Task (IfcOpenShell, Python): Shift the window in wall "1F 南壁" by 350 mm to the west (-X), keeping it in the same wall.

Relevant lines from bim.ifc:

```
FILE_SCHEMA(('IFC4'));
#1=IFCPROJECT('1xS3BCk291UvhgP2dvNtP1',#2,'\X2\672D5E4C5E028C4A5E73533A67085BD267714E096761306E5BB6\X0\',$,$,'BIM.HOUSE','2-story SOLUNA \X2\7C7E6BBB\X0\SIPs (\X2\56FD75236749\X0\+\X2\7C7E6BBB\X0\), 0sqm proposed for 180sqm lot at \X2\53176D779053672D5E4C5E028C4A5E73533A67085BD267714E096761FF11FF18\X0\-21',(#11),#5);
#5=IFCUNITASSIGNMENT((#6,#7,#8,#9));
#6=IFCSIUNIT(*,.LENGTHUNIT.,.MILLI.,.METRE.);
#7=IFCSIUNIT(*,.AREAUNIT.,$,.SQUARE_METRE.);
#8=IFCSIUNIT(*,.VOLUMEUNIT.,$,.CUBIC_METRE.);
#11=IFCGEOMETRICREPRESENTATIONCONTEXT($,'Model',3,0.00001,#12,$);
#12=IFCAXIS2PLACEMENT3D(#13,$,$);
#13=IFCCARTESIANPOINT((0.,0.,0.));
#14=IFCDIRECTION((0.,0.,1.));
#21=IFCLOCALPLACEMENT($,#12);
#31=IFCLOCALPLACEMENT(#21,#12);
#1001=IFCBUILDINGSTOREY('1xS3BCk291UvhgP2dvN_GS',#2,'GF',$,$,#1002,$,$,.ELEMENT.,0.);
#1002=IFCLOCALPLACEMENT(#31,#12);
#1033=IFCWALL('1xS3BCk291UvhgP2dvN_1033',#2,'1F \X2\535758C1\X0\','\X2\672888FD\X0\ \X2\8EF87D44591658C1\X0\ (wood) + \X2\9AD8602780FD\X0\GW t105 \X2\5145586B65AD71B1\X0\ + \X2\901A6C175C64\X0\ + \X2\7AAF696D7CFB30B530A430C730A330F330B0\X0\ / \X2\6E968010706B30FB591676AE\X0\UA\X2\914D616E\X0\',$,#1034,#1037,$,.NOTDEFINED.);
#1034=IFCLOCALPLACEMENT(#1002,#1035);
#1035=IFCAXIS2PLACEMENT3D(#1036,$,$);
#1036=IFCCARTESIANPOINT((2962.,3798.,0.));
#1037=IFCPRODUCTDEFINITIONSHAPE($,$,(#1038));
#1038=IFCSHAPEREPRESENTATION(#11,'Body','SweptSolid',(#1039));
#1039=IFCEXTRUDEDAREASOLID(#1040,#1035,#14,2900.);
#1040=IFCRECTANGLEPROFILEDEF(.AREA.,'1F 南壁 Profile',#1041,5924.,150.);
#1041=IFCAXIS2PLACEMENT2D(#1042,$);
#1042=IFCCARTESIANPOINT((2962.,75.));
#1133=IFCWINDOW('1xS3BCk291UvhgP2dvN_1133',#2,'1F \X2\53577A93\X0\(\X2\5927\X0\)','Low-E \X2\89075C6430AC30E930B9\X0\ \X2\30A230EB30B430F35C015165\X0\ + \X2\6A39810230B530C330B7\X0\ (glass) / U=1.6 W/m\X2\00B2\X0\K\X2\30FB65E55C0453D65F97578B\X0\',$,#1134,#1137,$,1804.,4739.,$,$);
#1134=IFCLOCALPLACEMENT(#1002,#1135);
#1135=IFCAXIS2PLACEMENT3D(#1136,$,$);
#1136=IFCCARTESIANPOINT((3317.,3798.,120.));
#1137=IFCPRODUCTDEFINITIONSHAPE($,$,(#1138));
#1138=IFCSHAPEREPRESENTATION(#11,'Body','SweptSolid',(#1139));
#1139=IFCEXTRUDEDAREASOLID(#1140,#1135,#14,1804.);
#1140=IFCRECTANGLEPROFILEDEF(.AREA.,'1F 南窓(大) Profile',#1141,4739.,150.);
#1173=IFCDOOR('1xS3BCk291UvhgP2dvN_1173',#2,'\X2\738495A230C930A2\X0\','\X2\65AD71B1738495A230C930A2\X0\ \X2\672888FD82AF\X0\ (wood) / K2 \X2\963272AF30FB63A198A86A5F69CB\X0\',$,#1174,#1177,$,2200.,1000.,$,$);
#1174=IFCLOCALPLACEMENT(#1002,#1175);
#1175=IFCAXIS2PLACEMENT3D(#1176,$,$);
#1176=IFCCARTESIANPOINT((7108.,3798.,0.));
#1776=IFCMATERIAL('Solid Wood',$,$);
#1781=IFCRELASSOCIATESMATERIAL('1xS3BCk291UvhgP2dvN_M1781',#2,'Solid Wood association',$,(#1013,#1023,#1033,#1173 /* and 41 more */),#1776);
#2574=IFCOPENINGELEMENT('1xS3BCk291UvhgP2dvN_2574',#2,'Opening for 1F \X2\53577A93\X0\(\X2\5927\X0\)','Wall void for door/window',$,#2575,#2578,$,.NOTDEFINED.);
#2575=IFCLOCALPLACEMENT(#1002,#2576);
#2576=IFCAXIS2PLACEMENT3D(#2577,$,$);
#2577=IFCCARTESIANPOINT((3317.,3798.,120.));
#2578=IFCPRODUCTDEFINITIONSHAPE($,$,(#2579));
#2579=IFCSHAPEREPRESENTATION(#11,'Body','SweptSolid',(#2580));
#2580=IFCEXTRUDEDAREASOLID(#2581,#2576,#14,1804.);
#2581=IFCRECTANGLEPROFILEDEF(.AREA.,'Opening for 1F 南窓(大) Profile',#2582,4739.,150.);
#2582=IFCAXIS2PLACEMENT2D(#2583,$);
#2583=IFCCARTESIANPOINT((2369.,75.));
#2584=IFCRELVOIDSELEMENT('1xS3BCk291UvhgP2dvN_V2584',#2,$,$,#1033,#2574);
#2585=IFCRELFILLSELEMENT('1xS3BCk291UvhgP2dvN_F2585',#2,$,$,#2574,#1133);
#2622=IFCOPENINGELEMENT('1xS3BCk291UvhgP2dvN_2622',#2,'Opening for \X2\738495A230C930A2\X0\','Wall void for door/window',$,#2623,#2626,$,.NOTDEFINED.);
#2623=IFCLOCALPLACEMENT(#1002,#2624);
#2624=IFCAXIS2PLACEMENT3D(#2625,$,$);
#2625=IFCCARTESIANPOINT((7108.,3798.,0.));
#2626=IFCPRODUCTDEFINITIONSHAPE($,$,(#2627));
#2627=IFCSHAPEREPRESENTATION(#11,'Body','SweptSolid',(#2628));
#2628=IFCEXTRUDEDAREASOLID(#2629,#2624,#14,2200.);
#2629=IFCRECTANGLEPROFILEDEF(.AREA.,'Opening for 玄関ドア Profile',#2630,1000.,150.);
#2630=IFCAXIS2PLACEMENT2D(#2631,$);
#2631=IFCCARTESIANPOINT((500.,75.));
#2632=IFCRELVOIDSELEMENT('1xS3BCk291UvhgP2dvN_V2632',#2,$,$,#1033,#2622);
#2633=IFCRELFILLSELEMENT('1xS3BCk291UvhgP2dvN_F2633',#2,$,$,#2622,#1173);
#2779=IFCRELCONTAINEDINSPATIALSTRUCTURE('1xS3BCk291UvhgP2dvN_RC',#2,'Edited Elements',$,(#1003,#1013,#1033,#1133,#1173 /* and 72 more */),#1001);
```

```python
import ifcopenshell
import ifcopenshell.api.geometry
import ifcopenshell.util.placement
import ifcopenshell.util.unit

model = ifcopenshell.open("bim.ifc")
unit_scale = ifcopenshell.util.unit.calculate_unit_scale(model)

window = model.by_id(1133)
opening = window.FillsVoids[0].RelatingOpeningElement
wall = opening.VoidsElements[0].RelatingBuildingElement

wall_matrix = ifcopenshell.util.placement.get_local_placement(wall.ObjectPlacement)
shift = wall_matrix[:3, 0] * -0.35 / unit_scale
before = ifcopenshell.util.placement.get_local_placement(window.ObjectPlacement)[:3, 3].copy()

# The window is not placed relative to its opening, so move both.
for product in (opening, window):
    matrix = ifcopenshell.util.placement.get_local_placement(product.ObjectPlacement)
    matrix[:3, 3] += shift
    ifcopenshell.api.geometry.edit_object_placement(model, product=product, matrix=matrix, is_si=False)

after = ifcopenshell.util.placement.get_local_placement(window.ObjectPlacement)[:3, 3]
print("window moved by", (after - before).round(3) + 0.0)

model.write("bim-out.ifc")
```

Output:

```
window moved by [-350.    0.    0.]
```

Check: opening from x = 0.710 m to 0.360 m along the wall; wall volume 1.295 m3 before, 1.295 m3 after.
